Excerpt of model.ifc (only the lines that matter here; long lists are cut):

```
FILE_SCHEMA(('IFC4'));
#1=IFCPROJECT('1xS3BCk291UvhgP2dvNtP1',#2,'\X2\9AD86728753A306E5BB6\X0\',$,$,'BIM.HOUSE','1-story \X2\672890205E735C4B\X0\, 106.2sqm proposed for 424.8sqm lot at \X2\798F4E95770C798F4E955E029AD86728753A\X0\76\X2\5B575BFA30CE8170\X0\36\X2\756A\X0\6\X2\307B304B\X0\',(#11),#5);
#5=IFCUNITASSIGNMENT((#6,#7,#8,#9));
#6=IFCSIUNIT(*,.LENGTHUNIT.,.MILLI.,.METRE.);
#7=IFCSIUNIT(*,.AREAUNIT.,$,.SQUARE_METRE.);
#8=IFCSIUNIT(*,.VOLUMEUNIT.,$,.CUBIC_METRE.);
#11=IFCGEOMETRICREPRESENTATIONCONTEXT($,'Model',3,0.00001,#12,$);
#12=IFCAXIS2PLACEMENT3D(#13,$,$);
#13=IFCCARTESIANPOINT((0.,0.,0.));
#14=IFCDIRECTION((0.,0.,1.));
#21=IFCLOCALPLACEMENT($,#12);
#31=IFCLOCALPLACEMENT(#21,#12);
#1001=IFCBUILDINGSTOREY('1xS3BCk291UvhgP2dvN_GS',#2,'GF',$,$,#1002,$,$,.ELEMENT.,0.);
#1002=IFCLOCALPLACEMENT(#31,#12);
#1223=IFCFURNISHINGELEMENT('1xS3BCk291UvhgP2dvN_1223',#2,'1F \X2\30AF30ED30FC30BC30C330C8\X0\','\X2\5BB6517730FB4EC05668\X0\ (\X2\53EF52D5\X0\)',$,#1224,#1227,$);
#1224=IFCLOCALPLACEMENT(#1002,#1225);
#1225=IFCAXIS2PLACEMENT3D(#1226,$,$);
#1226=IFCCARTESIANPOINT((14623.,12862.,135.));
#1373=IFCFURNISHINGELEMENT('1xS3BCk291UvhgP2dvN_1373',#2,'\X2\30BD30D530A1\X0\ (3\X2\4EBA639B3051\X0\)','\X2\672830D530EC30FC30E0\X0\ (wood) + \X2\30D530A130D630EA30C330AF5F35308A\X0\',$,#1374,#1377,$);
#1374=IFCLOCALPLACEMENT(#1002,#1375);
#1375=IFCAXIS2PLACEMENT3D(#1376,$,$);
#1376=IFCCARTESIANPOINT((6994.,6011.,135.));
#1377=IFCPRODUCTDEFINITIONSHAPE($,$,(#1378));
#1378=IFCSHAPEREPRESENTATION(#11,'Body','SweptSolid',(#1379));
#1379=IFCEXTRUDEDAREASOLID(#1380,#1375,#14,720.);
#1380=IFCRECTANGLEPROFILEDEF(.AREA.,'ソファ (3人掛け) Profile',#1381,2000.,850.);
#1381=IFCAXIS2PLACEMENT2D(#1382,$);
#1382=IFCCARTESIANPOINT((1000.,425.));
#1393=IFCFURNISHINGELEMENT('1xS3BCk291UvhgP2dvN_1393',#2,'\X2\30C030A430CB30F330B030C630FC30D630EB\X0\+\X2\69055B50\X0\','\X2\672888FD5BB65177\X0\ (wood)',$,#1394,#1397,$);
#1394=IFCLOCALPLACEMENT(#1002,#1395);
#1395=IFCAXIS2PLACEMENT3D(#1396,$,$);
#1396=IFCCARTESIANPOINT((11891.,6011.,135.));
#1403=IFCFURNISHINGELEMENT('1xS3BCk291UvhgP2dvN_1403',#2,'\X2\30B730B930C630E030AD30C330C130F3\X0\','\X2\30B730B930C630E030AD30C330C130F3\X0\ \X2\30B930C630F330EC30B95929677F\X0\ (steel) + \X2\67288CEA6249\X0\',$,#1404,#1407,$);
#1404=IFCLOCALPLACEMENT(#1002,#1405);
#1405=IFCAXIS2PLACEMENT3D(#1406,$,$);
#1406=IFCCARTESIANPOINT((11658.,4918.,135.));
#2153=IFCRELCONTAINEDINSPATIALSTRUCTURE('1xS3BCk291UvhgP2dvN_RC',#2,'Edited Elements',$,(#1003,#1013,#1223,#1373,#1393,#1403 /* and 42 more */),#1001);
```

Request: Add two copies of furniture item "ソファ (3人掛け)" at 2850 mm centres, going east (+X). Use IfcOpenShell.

```python
import numpy as np
import ifcopenshell
import ifcopenshell.api.geometry
import ifcopenshell.api.root
import ifcopenshell.util.element
import ifcopenshell.util.placement
import ifcopenshell.util.unit

model = ifcopenshell.open("model.ifc")
unit_scale = ifcopenshell.util.unit.calculate_unit_scale(model)


def reuse_history(source, copy):
    """copy_class also copies each property set's owner history, people and application; keep the originals."""
    for rel in copy.IsDefinedBy:
        if rel.is_a("IfcRelDefinesByProperties") and (history := rel.RelatingPropertyDefinition.OwnerHistory):
            rel.RelatingPropertyDefinition.OwnerHistory = source.OwnerHistory
            ifcopenshell.util.element.remove_deep2(model, history)


source = model.by_guid("1xS3BCk291UvhgP2dvN_1373")
base = ifcopenshell.util.placement.get_local_placement(source.ObjectPlacement)
step = np.array([1.0, 0.0, 0.0]) * 2.85 / unit_scale

for i in range(1, 3):
    copy = ifcopenshell.api.root.copy_class(model, product=source)
    copy.Representation = ifcopenshell.util.element.copy_deep(
        model, source.Representation, exclude=["IfcGeometricRepresentationContext", "IfcRepresentationMap"]
    )
    reuse_history(source, copy)
    matrix = base.copy()
    matrix[:3, 3] += i * step
    print("added at", matrix[:3, 3].round(3) + 0.0)
    ifcopenshell.api.geometry.edit_object_placement(model, product=copy, matrix=matrix, is_si=False)

model.write("model_edited.ifc")
```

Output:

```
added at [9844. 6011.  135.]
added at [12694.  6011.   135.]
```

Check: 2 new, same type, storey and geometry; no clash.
